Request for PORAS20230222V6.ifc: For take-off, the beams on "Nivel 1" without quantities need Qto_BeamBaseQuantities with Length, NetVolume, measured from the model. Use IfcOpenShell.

First a look at what the model holds.

```python
import ifcopenshell
import ifcopenshell.util.element
import ifcopenshell.util.unit

model = ifcopenshell.open("PORAS20230222V6.ifc")
print(model.schema)
for unit_type in ("LENGTHUNIT", "AREAUNIT", "VOLUMEUNIT"):
    print(unit_type, ifcopenshell.util.unit.calculate_unit_scale(model, unit_type))
storey = next(s for s in model.by_type("IfcBuildingStorey") if s.Name == "Nivel 1")
beams = [e for e in ifcopenshell.util.element.get_decomposition(storey) if e.is_a("IfcBeam")]
for e in sorted(beams, key=lambda e: e.id()):
    print(e.id(), e.is_a(), e.Name, list(ifcopenshell.util.element.get_psets(e, qtos_only=True)), sep=" | ")
```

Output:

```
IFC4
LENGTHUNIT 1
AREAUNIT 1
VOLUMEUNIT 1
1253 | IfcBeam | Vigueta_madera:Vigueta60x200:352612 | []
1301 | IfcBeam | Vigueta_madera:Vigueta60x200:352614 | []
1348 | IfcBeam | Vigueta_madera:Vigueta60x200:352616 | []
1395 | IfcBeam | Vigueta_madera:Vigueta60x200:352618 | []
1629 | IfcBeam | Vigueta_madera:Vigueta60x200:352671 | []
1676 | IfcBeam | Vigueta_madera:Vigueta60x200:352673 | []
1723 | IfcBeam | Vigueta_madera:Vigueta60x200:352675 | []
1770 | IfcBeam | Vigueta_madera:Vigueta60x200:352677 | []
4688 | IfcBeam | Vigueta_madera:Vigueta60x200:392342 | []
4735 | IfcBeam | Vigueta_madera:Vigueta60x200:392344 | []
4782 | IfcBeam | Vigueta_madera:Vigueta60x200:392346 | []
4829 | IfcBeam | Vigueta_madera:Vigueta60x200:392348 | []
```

```python
import ifcopenshell
import ifcopenshell.api.pset
import ifcopenshell.geom
import ifcopenshell.util.element
import ifcopenshell.util.shape
import ifcopenshell.util.unit

model = ifcopenshell.open("PORAS20230222V6.ifc")
unit_scale = ifcopenshell.util.unit.calculate_unit_scale(model)
volume_scale = ifcopenshell.util.unit.calculate_unit_scale(model, "VOLUMEUNIT")
settings = ifcopenshell.geom.settings()

storey = next(s for s in model.by_type("IfcBuildingStorey") if s.Name == "Nivel 1")
beams = [e for e in ifcopenshell.util.element.get_decomposition(storey) if e.is_a("IfcBeam")]

for e in sorted(beams, key=lambda e: e.id()):
    if ifcopenshell.util.element.get_psets(e, qtos_only=True, should_inherit=False):
        continue
    # Geometry comes back in metres, in the element's own axes.
    shape = ifcopenshell.geom.create_shape(settings, e)
    values = {
        "Length": ifcopenshell.util.shape.get_max_xyz(shape.geometry) / unit_scale,
        "NetVolume": ifcopenshell.util.shape.get_volume(shape.geometry) / volume_scale,
    }
    qto = ifcopenshell.api.pset.add_qto(model, product=e, name="Qto_BeamBaseQuantities")
    ifcopenshell.api.pset.edit_qto(model, qto=qto, properties=values)
    print(e.id(), {k: round(v, 3) for k, v in values.items()})

model.write("PORAS20230222V6_edited.ifc")
```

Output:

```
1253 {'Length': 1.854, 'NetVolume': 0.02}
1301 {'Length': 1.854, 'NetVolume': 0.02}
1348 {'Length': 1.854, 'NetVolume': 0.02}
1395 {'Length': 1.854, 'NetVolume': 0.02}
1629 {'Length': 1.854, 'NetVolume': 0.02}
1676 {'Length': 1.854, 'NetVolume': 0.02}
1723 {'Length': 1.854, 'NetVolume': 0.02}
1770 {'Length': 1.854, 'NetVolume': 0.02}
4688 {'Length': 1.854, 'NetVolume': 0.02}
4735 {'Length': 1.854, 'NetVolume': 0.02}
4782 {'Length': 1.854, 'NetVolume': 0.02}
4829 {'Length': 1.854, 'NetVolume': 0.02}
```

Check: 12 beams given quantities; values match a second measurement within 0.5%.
